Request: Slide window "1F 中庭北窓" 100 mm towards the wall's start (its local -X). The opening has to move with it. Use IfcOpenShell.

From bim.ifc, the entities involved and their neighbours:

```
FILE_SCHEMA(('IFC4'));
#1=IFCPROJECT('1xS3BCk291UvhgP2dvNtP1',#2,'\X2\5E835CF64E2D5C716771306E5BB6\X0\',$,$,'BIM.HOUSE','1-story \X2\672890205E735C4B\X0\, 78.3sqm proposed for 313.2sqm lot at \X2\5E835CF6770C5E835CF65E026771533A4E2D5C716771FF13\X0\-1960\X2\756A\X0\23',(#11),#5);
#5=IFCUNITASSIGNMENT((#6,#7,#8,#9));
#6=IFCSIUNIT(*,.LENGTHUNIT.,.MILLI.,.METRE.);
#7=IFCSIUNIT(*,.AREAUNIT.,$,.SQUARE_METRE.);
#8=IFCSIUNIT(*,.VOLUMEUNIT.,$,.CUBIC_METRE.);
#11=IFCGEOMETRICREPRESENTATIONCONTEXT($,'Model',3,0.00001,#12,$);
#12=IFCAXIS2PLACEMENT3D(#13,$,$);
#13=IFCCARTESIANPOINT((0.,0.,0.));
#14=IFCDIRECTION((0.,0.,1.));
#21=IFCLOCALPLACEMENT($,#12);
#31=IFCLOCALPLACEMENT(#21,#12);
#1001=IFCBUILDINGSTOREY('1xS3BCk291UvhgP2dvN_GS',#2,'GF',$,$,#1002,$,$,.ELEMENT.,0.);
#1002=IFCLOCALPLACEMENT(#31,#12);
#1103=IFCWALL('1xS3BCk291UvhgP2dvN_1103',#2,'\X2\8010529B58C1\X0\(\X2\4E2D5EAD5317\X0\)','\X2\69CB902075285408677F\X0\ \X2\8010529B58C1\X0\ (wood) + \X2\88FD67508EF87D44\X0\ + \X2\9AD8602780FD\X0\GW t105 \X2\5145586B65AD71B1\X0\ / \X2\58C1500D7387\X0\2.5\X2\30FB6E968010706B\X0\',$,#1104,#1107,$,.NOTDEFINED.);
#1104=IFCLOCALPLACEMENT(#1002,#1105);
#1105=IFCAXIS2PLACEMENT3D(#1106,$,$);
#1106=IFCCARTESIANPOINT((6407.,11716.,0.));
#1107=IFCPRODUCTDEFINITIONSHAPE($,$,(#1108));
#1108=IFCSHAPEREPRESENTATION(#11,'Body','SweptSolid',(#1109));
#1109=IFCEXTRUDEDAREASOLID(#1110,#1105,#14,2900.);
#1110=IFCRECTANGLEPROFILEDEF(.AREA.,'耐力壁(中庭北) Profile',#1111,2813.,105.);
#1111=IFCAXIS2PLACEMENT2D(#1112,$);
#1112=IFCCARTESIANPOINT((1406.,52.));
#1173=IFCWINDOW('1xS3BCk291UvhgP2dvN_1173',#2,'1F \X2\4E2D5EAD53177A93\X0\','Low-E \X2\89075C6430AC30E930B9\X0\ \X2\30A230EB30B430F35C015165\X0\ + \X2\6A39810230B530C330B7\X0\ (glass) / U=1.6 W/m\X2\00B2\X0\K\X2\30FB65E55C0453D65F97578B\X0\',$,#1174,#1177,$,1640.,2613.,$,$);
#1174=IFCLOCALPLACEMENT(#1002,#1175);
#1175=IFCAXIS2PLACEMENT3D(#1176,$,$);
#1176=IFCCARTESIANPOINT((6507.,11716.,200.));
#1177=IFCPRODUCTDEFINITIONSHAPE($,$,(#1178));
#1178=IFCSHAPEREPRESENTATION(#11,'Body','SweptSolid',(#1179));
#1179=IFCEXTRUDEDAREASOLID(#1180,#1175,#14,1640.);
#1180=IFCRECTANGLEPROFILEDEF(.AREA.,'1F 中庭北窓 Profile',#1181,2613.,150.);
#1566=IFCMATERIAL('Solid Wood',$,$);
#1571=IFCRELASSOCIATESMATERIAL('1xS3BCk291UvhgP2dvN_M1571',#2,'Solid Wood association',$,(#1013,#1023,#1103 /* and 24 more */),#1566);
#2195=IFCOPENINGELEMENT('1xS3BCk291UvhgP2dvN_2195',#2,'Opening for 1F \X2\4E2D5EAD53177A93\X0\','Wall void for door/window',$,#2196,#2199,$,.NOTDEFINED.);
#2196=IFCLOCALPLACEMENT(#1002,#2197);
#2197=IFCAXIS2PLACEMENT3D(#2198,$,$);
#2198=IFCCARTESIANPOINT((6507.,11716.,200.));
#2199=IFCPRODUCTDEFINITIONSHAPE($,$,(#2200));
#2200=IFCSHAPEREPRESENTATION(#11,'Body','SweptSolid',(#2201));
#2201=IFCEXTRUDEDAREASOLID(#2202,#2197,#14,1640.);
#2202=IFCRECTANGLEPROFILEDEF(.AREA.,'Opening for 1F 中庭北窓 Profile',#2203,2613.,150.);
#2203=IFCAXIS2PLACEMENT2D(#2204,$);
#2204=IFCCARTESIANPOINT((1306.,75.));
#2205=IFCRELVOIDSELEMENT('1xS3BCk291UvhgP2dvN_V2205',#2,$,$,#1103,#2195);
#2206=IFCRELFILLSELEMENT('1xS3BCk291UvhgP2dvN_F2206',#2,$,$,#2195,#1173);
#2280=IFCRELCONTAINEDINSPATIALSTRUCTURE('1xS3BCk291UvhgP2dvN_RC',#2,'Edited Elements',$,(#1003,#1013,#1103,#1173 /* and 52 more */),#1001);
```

```python
import ifcopenshell
import ifcopenshell.api.geometry
import ifcopenshell.util.placement
import ifcopenshell.util.unit

model = ifcopenshell.open("bim.ifc")
unit_scale = ifcopenshell.util.unit.calculate_unit_scale(model)

window = model.by_guid("1xS3BCk291UvhgP2dvN_1173")
opening = window.FillsVoids[0].RelatingOpeningElement
wall = opening.VoidsElements[0].RelatingBuildingElement

wall_matrix = ifcopenshell.util.placement.get_local_placement(wall.ObjectPlacement)
shift = wall_matrix[:3, 0] * -0.1 / unit_scale
before = ifcopenshell.util.placement.get_local_placement(window.ObjectPlacement)[:3, 3].copy()

# The window is not placed relative to its opening, so move both.
for product in (opening, window):
    matrix = ifcopenshell.util.placement.get_local_placement(product.ObjectPlacement)
    matrix[:3, 3] += shift
    ifcopenshell.api.geometry.edit_object_placement(model, product=product, matrix=matrix, is_si=False)

after = ifcopenshell.util.placement.get_local_placement(window.ObjectPlacement)[:3, 3]
print("window moved by", (after - before).round(3) + 0.0)

model.write("bim_edited.ifc")
```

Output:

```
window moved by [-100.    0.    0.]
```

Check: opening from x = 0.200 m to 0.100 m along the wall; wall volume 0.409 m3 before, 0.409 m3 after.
